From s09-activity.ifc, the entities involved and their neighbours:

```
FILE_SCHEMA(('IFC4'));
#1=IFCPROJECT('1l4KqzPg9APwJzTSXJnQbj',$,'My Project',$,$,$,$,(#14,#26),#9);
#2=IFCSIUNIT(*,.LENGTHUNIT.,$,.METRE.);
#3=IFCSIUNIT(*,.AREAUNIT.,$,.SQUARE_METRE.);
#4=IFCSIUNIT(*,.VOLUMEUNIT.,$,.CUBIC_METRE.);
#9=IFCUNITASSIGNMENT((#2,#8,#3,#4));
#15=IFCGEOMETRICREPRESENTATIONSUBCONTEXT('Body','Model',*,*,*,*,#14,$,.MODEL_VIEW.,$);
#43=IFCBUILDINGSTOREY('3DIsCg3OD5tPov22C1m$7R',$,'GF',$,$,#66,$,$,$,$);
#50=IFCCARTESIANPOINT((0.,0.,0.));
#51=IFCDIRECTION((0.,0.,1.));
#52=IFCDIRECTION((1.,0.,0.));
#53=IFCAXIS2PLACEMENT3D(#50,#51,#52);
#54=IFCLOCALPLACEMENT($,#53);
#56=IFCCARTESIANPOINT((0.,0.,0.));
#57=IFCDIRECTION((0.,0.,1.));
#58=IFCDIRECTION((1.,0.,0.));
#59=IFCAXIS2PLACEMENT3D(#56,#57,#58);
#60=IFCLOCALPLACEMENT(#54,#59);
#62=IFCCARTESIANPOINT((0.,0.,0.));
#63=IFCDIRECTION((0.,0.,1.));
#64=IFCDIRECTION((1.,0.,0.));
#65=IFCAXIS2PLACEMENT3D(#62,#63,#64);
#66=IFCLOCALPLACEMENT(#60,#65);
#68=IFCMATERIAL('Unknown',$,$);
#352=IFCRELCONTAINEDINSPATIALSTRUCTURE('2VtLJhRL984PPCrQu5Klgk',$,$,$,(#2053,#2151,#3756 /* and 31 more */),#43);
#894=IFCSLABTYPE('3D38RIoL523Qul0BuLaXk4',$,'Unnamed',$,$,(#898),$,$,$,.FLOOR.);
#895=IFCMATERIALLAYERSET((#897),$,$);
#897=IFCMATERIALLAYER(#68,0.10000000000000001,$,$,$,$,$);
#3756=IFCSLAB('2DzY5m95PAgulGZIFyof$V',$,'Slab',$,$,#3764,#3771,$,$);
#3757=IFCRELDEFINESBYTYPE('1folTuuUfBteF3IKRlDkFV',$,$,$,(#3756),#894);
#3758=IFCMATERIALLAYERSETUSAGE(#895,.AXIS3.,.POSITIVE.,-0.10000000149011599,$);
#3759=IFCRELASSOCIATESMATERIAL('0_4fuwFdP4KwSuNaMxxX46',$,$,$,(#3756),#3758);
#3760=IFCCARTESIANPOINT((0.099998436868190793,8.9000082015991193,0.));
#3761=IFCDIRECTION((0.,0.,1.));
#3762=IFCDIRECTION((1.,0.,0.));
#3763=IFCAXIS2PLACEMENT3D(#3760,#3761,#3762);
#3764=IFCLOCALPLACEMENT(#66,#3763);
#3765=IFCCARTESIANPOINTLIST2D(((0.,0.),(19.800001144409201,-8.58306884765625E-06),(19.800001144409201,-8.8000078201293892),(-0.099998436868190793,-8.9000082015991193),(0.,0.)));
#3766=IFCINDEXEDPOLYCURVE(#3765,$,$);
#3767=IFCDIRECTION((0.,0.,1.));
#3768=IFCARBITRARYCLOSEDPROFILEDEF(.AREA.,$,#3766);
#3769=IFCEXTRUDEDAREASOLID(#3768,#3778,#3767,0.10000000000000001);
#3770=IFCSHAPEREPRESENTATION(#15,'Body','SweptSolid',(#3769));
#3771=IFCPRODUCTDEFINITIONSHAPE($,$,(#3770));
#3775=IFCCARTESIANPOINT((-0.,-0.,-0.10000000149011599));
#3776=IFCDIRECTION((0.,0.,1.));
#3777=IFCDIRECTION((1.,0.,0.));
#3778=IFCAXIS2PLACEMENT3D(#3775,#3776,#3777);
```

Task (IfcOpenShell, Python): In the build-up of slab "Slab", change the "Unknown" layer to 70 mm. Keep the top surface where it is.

```python
import ifcopenshell
import ifcopenshell.util.element
import ifcopenshell.util.representation

model = ifcopenshell.open("s09-activity.ifc")

layer_set = model.by_id(895)
layer = next(l for l in layer_set.MaterialLayers if l.Material and l.Material.Name == "Unknown")
change = 0.07 - layer.LayerThickness
layer.LayerThickness += change

# Geometry does not follow the layer set by itself.
slabs = [e for e in ifcopenshell.util.element.get_elements_by_material(model, layer_set) if e.is_a("IfcSlab")]
for slab in sorted(slabs, key=lambda e: e.id()):
    body = ifcopenshell.util.representation.get_representation(slab, "Model", "Body")
    solid = body.Items[0]
    old_depth = solid.Depth
    solid.Depth += change
    # Extruded upwards: lower the start of the extrusion so the top stays.
    x, y, z = solid.Position.Location.Coordinates
    solid.Position.Location = model.createIfcCartesianPoint((x, y, z - change))
    print(slab.id(), f"{old_depth:g} -> {solid.Depth:g}")

# The layers are counted up from the underside, which has moved.
for usage in {ifcopenshell.util.element.get_material(slab) for slab in slabs}:
    usage.OffsetFromReferenceLine -= change

model.write("s09-activity_v2.ifc")
```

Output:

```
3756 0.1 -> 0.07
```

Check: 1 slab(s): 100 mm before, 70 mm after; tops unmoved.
